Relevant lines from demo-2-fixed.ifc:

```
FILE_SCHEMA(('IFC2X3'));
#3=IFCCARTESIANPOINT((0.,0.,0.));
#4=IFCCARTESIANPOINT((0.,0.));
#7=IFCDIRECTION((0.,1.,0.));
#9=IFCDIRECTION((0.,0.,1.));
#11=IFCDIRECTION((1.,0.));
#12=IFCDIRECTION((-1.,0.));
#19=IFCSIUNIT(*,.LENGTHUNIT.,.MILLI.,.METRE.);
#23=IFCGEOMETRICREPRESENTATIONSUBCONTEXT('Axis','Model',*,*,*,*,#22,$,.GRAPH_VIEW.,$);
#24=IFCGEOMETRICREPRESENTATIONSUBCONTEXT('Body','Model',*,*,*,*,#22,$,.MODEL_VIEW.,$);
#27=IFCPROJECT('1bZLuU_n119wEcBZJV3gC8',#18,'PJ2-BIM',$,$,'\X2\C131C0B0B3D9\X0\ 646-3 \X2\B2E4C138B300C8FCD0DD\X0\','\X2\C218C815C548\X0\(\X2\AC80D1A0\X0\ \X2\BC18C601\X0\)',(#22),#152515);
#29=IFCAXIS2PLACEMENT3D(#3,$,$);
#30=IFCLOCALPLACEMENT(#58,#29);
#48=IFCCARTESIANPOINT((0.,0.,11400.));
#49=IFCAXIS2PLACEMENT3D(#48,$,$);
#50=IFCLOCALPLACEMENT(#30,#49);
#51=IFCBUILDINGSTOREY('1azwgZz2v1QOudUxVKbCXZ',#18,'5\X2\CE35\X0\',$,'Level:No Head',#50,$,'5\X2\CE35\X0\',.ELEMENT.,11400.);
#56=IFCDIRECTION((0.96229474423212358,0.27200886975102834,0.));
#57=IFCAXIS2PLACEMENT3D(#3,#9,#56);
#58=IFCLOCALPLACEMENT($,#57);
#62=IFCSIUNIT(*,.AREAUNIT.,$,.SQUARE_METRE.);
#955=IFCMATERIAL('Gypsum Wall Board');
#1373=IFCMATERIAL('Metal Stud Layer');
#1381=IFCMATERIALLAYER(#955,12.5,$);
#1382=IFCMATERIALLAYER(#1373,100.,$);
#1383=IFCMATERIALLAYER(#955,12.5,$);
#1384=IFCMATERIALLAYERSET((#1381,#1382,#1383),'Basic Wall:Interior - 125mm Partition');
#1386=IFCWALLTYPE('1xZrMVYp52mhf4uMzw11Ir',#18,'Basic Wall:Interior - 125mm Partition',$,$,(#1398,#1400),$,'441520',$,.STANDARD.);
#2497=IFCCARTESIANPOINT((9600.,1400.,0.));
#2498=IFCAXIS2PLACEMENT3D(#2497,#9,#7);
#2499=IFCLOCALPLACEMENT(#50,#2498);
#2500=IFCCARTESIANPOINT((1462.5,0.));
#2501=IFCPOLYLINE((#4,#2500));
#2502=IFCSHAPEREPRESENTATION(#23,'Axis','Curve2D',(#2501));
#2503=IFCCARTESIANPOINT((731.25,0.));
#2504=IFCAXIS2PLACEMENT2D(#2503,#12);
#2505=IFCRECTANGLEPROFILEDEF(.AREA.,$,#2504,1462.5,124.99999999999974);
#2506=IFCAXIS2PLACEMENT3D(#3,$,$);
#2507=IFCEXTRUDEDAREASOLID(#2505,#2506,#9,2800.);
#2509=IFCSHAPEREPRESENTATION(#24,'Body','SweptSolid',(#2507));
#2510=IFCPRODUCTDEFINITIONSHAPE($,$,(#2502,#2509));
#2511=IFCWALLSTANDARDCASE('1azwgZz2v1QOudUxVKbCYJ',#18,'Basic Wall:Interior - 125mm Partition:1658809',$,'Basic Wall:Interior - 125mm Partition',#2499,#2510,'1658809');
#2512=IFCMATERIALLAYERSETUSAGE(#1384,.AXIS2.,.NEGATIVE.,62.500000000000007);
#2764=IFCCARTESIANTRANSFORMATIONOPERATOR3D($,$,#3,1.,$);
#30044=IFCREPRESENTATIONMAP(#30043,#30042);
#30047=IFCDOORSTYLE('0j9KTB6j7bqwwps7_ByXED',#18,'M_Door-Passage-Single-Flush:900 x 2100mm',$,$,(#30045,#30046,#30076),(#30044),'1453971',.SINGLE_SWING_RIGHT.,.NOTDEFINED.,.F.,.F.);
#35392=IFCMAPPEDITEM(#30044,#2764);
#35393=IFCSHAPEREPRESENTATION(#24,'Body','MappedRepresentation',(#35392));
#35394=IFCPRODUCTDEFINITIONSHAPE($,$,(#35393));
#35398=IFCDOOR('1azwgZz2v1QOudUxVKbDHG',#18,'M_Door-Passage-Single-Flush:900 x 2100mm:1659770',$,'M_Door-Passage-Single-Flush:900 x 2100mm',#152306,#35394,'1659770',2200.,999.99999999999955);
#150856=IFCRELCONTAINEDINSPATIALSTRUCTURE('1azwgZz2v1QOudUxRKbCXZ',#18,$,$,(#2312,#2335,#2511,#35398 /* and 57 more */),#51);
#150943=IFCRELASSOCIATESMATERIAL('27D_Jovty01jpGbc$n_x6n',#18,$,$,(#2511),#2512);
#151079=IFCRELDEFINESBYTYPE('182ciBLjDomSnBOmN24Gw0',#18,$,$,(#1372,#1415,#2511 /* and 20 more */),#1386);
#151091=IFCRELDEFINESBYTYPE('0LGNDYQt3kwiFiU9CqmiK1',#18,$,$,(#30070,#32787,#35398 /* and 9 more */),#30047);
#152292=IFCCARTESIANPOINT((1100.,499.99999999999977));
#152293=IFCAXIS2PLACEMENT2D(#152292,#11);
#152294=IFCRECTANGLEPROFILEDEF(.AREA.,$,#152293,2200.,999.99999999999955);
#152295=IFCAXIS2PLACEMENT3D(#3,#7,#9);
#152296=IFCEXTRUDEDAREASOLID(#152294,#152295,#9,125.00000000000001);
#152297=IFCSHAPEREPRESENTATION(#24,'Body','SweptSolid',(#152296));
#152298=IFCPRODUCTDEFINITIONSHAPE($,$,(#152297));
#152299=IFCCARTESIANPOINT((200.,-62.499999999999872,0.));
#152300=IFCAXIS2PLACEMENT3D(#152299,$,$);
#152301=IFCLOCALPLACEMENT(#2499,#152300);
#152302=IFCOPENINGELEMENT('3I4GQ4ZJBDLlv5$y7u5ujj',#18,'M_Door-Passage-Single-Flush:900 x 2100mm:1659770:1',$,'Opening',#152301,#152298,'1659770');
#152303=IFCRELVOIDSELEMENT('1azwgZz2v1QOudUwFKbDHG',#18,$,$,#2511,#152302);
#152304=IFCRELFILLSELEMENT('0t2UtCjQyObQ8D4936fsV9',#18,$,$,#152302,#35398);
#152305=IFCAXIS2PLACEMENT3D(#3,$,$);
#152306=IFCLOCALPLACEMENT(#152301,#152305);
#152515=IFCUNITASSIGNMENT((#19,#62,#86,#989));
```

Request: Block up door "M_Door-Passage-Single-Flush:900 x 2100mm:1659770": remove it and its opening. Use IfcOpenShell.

```python
import ifcopenshell
import ifcopenshell.api.feature
import ifcopenshell.api.root
import ifcopenshell.geom
import ifcopenshell.util.shape

model = ifcopenshell.open("demo-2-fixed.ifc")
settings = ifcopenshell.geom.settings()


def volume(element):
    """Net volume in cubic metres, openings subtracted."""
    shape = ifcopenshell.geom.create_shape(settings, element)
    return ifcopenshell.util.shape.get_volume(shape.geometry)


door = model.by_guid("1azwgZz2v1QOudUxVKbDHG")
opening = door.FillsVoids[0].RelatingOpeningElement
wall = opening.VoidsElements[0].RelatingBuildingElement
before = volume(wall)

ifcopenshell.api.root.remove_product(model, product=door)
ifcopenshell.api.feature.remove_feature(model, feature=opening)

after = volume(wall)

print(f"wall volume {before:.3f} -> {after:.3f} m3")

model.write("demo-2-fixed_edited.ifc")
```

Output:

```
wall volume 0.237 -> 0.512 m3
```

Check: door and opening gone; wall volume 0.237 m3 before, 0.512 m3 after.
